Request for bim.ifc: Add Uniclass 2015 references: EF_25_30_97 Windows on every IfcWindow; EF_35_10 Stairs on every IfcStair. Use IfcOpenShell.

First a look at what the model holds.

```python
import ifcopenshell

model = ifcopenshell.open("bim.ifc")
print(model.schema)
print("classifications:", [c.Name for c in model.by_type("IfcClassification")])
for ifc_class in ("IfcDoor", "IfcRoof", "IfcStair", "IfcWall", "IfcWindow"):
    print(ifc_class, len(model.by_type(ifc_class)))
```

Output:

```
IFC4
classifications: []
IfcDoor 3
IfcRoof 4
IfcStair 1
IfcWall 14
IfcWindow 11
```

```python
import ifcopenshell
import ifcopenshell.api.classification

model = ifcopenshell.open("bim.ifc")

system = ifcopenshell.api.classification.add_classification(model, classification="Uniclass 2015")

codes = {
    "IfcWindow": ("EF_25_30_97", "Windows"),
    "IfcStair": ("EF_35_10", "Stairs"),
}
for ifc_class, (code, name) in codes.items():
    products = model.by_type(ifc_class)
    ifcopenshell.api.classification.add_reference(
        model, products=products, classification=system, identification=code, name=name
    )
    print(code, len(products))

model.write("bim_updated.ifc")
```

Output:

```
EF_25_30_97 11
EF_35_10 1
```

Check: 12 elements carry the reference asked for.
